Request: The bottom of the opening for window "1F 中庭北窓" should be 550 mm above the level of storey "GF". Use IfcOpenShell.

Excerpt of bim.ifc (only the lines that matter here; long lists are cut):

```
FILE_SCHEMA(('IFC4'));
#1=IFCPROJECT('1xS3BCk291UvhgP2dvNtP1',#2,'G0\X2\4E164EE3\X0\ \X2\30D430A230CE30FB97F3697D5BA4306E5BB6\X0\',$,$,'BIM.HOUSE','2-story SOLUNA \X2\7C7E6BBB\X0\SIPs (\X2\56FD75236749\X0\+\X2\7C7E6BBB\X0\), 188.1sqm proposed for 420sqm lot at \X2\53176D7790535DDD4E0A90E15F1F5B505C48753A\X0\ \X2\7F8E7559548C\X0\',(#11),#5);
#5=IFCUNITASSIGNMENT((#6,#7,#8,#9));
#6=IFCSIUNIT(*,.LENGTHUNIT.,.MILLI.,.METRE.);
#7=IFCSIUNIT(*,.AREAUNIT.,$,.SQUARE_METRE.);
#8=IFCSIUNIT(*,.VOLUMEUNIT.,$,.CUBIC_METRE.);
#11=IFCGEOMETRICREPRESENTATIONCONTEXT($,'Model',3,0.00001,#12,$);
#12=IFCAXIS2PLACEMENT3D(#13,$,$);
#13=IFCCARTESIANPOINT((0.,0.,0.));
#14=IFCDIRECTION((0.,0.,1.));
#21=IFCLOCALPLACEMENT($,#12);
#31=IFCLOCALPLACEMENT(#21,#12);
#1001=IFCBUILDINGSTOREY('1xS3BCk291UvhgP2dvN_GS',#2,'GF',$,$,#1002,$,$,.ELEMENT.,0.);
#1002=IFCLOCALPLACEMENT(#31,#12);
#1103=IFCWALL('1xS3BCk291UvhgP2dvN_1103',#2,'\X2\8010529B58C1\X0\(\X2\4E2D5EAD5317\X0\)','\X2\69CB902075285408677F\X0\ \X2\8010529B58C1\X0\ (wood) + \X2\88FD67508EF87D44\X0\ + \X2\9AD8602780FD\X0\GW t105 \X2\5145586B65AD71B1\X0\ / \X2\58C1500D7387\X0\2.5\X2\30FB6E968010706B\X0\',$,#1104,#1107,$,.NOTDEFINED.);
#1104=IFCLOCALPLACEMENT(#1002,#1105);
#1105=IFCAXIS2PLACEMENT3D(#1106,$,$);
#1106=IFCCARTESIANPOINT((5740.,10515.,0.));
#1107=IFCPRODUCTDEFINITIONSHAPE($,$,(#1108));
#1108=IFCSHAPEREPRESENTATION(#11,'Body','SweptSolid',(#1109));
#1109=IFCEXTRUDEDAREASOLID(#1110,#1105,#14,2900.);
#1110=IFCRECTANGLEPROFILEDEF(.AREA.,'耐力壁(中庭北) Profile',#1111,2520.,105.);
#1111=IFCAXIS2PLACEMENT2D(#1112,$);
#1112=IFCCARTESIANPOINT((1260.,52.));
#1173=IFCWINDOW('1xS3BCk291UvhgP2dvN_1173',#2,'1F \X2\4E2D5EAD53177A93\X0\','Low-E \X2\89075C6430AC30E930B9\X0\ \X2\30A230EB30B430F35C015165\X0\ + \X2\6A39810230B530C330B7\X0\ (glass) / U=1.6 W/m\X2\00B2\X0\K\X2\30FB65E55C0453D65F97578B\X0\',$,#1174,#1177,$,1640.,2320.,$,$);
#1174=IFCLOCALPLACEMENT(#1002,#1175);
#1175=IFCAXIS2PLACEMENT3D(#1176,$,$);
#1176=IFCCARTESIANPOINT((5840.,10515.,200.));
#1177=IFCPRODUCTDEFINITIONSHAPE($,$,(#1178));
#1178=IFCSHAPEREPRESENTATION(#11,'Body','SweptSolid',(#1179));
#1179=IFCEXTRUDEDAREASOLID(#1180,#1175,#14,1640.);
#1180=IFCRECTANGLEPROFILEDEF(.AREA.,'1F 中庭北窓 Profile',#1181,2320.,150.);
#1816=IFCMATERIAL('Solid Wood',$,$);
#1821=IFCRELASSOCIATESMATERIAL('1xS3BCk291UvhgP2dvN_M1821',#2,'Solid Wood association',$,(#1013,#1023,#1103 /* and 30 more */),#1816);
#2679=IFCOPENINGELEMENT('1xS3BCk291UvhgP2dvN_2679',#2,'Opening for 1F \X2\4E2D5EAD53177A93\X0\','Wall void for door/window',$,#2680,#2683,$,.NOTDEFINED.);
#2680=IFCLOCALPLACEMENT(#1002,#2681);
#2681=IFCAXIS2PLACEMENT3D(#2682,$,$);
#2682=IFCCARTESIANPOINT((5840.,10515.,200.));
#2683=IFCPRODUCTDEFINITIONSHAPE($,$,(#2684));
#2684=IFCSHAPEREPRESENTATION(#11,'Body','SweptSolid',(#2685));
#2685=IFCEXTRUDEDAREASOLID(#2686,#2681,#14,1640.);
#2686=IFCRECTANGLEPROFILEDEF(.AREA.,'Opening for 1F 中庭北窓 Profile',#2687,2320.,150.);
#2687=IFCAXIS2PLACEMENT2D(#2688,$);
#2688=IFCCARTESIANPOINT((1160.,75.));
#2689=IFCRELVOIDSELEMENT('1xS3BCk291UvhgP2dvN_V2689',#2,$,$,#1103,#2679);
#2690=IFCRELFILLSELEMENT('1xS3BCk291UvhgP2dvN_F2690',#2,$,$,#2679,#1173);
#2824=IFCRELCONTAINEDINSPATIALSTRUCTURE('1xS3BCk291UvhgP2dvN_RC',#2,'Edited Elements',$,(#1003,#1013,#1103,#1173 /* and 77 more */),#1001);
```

```python
import numpy as np
import ifcopenshell
import ifcopenshell.api.geometry
import ifcopenshell.geom
import ifcopenshell.util.element
import ifcopenshell.util.placement
import ifcopenshell.util.shape
import ifcopenshell.util.unit

model = ifcopenshell.open("bim.ifc")
unit_scale = ifcopenshell.util.unit.calculate_unit_scale(model)

window = model.by_id(1173)
opening = window.FillsVoids[0].RelatingOpeningElement
storey = ifcopenshell.util.element.get_container(window, ifc_class="IfcBuildingStorey")
level = ifcopenshell.util.placement.get_local_placement(storey.ObjectPlacement)[2, 3]

# The opening's origin need not be at the sill, so measure its lowest point.
shape = ifcopenshell.geom.create_shape(ifcopenshell.geom.settings(), opening)
bottom = ifcopenshell.util.shape.get_shape_bottom_elevation(shape, shape.geometry) / unit_scale
dz = level + 550.0 - bottom

shift = np.array([0.0, 0.0, dz])
# The window is not placed relative to its opening, so move both.
for product in (opening, window):
    matrix = ifcopenshell.util.placement.get_local_placement(product.ObjectPlacement)
    matrix[:3, 3] += shift
    ifcopenshell.api.geometry.edit_object_placement(model, product=product, matrix=matrix, is_si=False)

print(f"moved by {dz * unit_scale:+.3f} m")

model.write("bim_rev.ifc")
```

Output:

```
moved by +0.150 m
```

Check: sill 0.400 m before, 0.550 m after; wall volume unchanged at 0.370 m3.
